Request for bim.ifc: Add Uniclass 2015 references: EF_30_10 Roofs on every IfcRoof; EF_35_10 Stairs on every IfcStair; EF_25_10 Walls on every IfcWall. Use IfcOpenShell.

First a look at what the model holds.

```python
import ifcopenshell

model = ifcopenshell.open("bim.ifc")
print(model.schema)
print("classifications:", [c.Name for c in model.by_type("IfcClassification")])
for ifc_class in ("IfcDoor", "IfcRoof", "IfcStair", "IfcWall", "IfcWindow"):
    print(ifc_class, len(model.by_type(ifc_class)))
```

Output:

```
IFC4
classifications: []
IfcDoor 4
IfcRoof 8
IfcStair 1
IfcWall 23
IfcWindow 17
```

```python
import ifcopenshell
import ifcopenshell.api.classification

model = ifcopenshell.open("bim.ifc")

system = ifcopenshell.api.classification.add_classification(model, classification="Uniclass 2015")

codes = {
    "IfcRoof": ("EF_30_10", "Roofs"),
    "IfcStair": ("EF_35_10", "Stairs"),
    "IfcWall": ("EF_25_10", "Walls"),
}
for ifc_class, (code, name) in codes.items():
    products = model.by_type(ifc_class)
    ifcopenshell.api.classification.add_reference(
        model, products=products, classification=system, identification=code, name=name
    )
    print(code, len(products))

model.write("bim_edited.ifc")
```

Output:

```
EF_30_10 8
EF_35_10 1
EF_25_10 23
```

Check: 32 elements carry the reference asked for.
